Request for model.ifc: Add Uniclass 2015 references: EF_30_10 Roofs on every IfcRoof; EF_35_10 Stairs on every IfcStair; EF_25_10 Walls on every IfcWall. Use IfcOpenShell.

First a look at what the model holds.

```python
import ifcopenshell

model = ifcopenshell.open("model.ifc")
print(model.schema)
print("classifications:", [c.Name for c in model.by_type("IfcClassification")])
for ifc_class in ("IfcDoor", "IfcRoof", "IfcStair", "IfcWall", "IfcWindow"):
    print(ifc_class, len(model.by_type(ifc_class)))
```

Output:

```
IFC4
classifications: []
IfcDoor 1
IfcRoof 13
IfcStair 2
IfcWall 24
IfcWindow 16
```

```python
import ifcopenshell
import ifcopenshell.api.classification

model = ifcopenshell.open("model.ifc")

system = ifcopenshell.api.classification.add_classification(model, classification="Uniclass 2015")

codes = {
    "IfcRoof": ("EF_30_10", "Roofs"),
    "IfcStair": ("EF_35_10", "Stairs"),
    "IfcWall": ("EF_25_10", "Walls"),
}
for ifc_class, (code, name) in codes.items():
    products = model.by_type(ifc_class)
    ifcopenshell.api.classification.add_reference(
        model, products=products, classification=system, identification=code, name=name
    )
    print(code, len(products))

model.write("model-out.ifc")
```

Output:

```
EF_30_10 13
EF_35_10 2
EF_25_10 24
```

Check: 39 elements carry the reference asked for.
